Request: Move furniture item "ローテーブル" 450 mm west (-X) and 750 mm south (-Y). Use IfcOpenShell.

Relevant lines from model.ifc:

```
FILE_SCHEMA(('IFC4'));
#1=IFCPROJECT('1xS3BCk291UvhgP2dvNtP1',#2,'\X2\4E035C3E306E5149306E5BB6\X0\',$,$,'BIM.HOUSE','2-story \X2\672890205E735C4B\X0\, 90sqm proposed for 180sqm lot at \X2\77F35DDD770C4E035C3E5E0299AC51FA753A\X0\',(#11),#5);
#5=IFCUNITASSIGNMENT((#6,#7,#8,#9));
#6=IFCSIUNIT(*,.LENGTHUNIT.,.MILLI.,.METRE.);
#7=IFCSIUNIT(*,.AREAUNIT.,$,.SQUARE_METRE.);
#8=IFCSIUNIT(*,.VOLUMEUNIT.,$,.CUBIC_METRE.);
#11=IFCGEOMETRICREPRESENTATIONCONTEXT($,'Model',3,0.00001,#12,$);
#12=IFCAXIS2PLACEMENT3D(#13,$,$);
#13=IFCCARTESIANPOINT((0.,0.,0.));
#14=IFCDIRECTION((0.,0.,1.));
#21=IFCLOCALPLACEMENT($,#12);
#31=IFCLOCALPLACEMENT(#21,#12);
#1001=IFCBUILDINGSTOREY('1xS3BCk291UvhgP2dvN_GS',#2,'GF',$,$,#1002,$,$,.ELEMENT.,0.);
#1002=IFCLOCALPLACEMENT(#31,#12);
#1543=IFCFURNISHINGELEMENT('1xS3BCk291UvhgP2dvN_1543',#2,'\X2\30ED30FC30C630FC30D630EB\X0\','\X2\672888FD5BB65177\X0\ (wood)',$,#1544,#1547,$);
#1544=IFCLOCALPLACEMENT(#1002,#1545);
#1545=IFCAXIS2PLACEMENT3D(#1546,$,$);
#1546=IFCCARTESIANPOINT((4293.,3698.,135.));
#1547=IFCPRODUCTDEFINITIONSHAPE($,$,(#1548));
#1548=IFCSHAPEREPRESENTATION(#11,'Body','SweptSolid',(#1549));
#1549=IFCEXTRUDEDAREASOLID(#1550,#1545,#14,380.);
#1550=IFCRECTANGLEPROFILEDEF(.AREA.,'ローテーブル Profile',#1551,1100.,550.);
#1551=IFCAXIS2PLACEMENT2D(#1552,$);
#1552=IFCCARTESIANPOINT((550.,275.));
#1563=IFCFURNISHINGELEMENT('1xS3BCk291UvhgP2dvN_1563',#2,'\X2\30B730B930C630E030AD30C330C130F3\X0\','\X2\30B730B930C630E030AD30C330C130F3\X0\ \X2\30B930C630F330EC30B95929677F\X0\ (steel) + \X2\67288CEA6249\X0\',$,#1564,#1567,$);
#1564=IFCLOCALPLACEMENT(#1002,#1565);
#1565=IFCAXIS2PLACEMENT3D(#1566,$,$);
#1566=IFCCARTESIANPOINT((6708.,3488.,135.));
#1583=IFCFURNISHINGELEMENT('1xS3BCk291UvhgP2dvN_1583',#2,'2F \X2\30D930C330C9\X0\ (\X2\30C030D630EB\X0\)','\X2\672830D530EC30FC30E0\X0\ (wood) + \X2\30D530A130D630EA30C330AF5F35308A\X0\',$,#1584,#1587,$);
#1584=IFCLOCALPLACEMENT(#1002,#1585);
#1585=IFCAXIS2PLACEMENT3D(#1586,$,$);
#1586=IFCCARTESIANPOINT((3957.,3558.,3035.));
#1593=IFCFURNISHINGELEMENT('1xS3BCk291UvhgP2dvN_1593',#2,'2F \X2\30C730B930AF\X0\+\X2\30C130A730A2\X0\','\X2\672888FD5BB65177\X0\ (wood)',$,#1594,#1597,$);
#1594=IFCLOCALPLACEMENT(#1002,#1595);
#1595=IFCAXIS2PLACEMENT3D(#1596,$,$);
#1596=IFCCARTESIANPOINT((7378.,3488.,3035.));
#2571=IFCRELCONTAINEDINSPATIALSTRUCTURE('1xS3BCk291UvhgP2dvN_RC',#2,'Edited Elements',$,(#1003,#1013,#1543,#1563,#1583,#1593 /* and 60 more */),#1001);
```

```python
import ifcopenshell
import ifcopenshell.api.geometry
import ifcopenshell.util.placement

model = ifcopenshell.open("model.ifc")

item = model.by_id(1543)
matrix = ifcopenshell.util.placement.get_local_placement(item.ObjectPlacement)
matrix[0, 3] -= 450.0
matrix[1, 3] -= 750.0
ifcopenshell.api.geometry.edit_object_placement(model, product=item, matrix=matrix, is_si=False)

print(ifcopenshell.util.placement.get_local_placement(item.ObjectPlacement).round(3) + 0.0)

model.write("model_v2.ifc")
```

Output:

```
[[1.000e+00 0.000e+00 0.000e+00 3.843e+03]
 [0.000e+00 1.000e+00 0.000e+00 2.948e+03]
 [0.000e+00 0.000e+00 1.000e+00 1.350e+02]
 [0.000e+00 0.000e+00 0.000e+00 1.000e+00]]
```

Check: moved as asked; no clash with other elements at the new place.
